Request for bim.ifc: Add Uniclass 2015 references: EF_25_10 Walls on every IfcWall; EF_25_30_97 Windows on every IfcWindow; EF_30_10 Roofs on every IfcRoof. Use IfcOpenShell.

First a look at what the model holds.

```python
import ifcopenshell

model = ifcopenshell.open("bim.ifc")
print(model.schema)
print("classifications:", [c.Name for c in model.by_type("IfcClassification")])
for ifc_class in ("IfcDoor", "IfcRoof", "IfcStair", "IfcWall", "IfcWindow"):
    print(ifc_class, len(model.by_type(ifc_class)))
```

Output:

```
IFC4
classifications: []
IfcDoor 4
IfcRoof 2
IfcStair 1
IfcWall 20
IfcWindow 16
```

```python
import ifcopenshell
import ifcopenshell.api.classification

model = ifcopenshell.open("bim.ifc")

system = ifcopenshell.api.classification.add_classification(model, classification="Uniclass 2015")

codes = {
    "IfcWall": ("EF_25_10", "Walls"),
    "IfcWindow": ("EF_25_30_97", "Windows"),
    "IfcRoof": ("EF_30_10", "Roofs"),
}
for ifc_class, (code, name) in codes.items():
    products = model.by_type(ifc_class)
    ifcopenshell.api.classification.add_reference(
        model, products=products, classification=system, identification=code, name=name
    )
    print(code, len(products))

model.write("bim_updated.ifc")
```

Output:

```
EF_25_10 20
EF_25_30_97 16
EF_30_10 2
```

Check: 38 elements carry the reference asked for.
